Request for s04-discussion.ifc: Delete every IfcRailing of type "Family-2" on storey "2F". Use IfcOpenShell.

First a look at what the model holds.

```python
import ifcopenshell
import ifcopenshell.util.element

model = ifcopenshell.open("s04-discussion.ifc")
print(model.schema)
storey = next(s for s in model.by_type("IfcBuildingStorey") if s.Name == "2F")
railings = [e for e in ifcopenshell.util.element.get_decomposition(storey) if e.is_a("IfcRailing")]
seen = {}
for e in railings:
    element_type = ifcopenshell.util.element.get_type(e)
    name = element_type.Name if element_type not in (None, e) else None
    seen[name] = seen.get(name, 0) + 1
for name, count in sorted(seen.items(), key=str):
    print(count, "x", name)
```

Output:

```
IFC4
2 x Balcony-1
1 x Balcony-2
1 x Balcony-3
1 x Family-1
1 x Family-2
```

```python
import ifcopenshell
import ifcopenshell.api.root
import ifcopenshell.util.element

model = ifcopenshell.open("s04-discussion.ifc")

storey = next(s for s in model.by_type("IfcBuildingStorey") if s.Name == "2F")
railings = [e for e in ifcopenshell.util.element.get_decomposition(storey) if e.is_a("IfcRailing")]
targets = [e for e in railings if (t := ifcopenshell.util.element.get_type(e)) not in (None, e) and t.Name == "Family-2"]

for e in targets:
    ifcopenshell.api.root.remove_product(model, product=e)
print(len(targets), "removed")

model.write("s04-discussion_rev.ifc")
```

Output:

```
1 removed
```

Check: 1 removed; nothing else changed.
